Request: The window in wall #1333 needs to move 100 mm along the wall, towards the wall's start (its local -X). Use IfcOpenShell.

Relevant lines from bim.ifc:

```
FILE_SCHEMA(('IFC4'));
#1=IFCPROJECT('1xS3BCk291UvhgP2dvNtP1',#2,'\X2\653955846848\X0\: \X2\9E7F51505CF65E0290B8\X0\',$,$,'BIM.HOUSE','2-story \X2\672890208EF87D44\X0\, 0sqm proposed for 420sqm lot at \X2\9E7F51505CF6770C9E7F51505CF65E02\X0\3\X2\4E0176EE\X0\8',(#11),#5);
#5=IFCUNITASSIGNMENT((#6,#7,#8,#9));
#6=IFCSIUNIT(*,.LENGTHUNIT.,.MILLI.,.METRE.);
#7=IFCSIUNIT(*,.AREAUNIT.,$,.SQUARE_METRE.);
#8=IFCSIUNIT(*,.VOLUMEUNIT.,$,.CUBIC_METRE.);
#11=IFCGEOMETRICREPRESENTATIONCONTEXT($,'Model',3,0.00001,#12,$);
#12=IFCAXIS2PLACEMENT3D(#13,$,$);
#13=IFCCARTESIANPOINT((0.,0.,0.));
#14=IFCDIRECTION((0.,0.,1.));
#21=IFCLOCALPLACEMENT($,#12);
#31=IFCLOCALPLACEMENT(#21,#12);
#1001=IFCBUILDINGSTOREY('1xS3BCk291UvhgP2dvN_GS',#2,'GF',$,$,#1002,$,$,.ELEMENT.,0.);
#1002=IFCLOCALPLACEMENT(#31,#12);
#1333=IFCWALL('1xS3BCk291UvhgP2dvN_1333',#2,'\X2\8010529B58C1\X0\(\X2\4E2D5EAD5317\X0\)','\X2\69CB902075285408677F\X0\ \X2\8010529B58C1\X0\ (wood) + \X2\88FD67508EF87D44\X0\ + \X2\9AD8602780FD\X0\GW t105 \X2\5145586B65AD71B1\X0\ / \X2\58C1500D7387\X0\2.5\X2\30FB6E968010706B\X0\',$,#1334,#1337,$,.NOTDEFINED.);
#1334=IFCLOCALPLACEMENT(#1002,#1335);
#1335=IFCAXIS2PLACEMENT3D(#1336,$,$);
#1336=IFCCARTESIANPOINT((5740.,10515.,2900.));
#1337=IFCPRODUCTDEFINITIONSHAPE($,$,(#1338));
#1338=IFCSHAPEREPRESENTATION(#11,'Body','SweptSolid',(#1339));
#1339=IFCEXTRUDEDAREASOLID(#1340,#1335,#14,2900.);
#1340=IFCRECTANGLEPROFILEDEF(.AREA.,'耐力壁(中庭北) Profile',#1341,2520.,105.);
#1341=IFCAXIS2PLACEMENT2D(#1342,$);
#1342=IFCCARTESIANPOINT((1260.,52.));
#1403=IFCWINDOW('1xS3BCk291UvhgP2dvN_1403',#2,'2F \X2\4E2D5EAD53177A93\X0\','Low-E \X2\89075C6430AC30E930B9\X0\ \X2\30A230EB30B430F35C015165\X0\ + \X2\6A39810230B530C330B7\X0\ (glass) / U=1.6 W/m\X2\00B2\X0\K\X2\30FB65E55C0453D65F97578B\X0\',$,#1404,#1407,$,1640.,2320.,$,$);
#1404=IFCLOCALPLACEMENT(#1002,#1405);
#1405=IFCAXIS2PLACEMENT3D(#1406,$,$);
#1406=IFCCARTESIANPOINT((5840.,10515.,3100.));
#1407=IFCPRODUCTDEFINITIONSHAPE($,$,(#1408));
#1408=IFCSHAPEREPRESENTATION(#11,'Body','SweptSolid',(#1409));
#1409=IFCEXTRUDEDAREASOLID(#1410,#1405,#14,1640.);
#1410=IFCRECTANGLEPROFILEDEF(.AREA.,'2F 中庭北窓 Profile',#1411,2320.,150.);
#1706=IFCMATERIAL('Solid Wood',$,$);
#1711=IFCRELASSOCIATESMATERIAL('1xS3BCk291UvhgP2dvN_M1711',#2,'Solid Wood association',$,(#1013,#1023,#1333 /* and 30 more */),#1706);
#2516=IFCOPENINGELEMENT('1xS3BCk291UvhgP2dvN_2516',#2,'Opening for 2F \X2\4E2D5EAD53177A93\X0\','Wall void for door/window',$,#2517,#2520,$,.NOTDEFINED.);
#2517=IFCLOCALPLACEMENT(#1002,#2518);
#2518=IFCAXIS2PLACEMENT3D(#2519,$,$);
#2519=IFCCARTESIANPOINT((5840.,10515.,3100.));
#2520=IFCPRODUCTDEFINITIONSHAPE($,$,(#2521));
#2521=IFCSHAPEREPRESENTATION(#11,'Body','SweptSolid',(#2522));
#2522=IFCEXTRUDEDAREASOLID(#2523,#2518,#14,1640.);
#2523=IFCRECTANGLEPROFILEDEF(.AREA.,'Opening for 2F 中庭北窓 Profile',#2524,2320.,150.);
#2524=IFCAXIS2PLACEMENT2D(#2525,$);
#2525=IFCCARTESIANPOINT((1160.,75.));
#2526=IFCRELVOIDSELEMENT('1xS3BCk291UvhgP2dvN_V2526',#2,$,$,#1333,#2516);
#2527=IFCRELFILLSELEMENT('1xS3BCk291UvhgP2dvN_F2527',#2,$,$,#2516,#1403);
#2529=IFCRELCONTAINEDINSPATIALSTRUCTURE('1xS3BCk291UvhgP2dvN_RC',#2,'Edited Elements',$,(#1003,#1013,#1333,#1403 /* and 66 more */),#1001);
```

```python
import ifcopenshell
import ifcopenshell.api.geometry
import ifcopenshell.util.placement
import ifcopenshell.util.unit

model = ifcopenshell.open("bim.ifc")
unit_scale = ifcopenshell.util.unit.calculate_unit_scale(model)

window = model.by_id(1403)
opening = window.FillsVoids[0].RelatingOpeningElement
wall = opening.VoidsElements[0].RelatingBuildingElement

wall_matrix = ifcopenshell.util.placement.get_local_placement(wall.ObjectPlacement)
shift = wall_matrix[:3, 0] * -0.1 / unit_scale
before = ifcopenshell.util.placement.get_local_placement(window.ObjectPlacement)[:3, 3].copy()

# The window is not placed relative to its opening, so move both.
for product in (opening, window):
    matrix = ifcopenshell.util.placement.get_local_placement(product.ObjectPlacement)
    matrix[:3, 3] += shift
    ifcopenshell.api.geometry.edit_object_placement(model, product=product, matrix=matrix, is_si=False)

after = ifcopenshell.util.placement.get_local_placement(window.ObjectPlacement)[:3, 3]
print("window moved by", (after - before).round(3) + 0.0)

model.write("bim_rev.ifc")
```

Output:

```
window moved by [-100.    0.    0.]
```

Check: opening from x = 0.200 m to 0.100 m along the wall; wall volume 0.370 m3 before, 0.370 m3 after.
